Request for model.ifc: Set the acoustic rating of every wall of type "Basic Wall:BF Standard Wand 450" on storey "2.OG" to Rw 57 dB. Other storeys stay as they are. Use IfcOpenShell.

First a look at what the model holds.

```python
import ifcopenshell
import ifcopenshell.util.element

model = ifcopenshell.open("model.ifc")
print(model.schema)
storey = next(s for s in model.by_type("IfcBuildingStorey") if s.Name == "2.OG")
walls = [e for e in ifcopenshell.util.element.get_decomposition(storey) if e.is_a("IfcWall")]
seen = {}
for e in walls:
    element_type = ifcopenshell.util.element.get_type(e)
    key = (element_type.Name if element_type != e and element_type else None, ifcopenshell.util.element.get_pset(e, "Pset_WallCommon", "AcousticRating"))
    seen[key] = seen.get(key, 0) + 1
for (name, value), count in sorted(seen.items(), key=str):
    print(count, "x", name, "|", value)
```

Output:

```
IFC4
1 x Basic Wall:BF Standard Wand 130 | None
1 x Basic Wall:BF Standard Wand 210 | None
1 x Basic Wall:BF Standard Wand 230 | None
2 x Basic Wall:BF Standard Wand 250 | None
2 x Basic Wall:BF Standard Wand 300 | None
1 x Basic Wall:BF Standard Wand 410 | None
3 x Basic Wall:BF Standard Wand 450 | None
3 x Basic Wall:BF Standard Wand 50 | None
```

```python
import ifcopenshell
import ifcopenshell.api.pset
import ifcopenshell.util.element

model = ifcopenshell.open("model.ifc")

storey = next(s for s in model.by_type("IfcBuildingStorey") if s.Name == "2.OG")
walls = [e for e in ifcopenshell.util.element.get_decomposition(storey) if e.is_a("IfcWall")]

count = 0
for e in walls:
    element_type = ifcopenshell.util.element.get_type(e)
    if element_type in (None, e) or element_type.Name != "Basic Wall:BF Standard Wand 450":
        continue
    # add_pset returns the element's existing set when there is one.
    pset = ifcopenshell.api.pset.add_pset(model, product=e, name="Pset_WallCommon")
    ifcopenshell.api.pset.edit_pset(model, pset=pset, properties={"AcousticRating": "Rw 57 dB"})
    count += 1

print(count, "walls updated")

model.write("model_rev.ifc")
```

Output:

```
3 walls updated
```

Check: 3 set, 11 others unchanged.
